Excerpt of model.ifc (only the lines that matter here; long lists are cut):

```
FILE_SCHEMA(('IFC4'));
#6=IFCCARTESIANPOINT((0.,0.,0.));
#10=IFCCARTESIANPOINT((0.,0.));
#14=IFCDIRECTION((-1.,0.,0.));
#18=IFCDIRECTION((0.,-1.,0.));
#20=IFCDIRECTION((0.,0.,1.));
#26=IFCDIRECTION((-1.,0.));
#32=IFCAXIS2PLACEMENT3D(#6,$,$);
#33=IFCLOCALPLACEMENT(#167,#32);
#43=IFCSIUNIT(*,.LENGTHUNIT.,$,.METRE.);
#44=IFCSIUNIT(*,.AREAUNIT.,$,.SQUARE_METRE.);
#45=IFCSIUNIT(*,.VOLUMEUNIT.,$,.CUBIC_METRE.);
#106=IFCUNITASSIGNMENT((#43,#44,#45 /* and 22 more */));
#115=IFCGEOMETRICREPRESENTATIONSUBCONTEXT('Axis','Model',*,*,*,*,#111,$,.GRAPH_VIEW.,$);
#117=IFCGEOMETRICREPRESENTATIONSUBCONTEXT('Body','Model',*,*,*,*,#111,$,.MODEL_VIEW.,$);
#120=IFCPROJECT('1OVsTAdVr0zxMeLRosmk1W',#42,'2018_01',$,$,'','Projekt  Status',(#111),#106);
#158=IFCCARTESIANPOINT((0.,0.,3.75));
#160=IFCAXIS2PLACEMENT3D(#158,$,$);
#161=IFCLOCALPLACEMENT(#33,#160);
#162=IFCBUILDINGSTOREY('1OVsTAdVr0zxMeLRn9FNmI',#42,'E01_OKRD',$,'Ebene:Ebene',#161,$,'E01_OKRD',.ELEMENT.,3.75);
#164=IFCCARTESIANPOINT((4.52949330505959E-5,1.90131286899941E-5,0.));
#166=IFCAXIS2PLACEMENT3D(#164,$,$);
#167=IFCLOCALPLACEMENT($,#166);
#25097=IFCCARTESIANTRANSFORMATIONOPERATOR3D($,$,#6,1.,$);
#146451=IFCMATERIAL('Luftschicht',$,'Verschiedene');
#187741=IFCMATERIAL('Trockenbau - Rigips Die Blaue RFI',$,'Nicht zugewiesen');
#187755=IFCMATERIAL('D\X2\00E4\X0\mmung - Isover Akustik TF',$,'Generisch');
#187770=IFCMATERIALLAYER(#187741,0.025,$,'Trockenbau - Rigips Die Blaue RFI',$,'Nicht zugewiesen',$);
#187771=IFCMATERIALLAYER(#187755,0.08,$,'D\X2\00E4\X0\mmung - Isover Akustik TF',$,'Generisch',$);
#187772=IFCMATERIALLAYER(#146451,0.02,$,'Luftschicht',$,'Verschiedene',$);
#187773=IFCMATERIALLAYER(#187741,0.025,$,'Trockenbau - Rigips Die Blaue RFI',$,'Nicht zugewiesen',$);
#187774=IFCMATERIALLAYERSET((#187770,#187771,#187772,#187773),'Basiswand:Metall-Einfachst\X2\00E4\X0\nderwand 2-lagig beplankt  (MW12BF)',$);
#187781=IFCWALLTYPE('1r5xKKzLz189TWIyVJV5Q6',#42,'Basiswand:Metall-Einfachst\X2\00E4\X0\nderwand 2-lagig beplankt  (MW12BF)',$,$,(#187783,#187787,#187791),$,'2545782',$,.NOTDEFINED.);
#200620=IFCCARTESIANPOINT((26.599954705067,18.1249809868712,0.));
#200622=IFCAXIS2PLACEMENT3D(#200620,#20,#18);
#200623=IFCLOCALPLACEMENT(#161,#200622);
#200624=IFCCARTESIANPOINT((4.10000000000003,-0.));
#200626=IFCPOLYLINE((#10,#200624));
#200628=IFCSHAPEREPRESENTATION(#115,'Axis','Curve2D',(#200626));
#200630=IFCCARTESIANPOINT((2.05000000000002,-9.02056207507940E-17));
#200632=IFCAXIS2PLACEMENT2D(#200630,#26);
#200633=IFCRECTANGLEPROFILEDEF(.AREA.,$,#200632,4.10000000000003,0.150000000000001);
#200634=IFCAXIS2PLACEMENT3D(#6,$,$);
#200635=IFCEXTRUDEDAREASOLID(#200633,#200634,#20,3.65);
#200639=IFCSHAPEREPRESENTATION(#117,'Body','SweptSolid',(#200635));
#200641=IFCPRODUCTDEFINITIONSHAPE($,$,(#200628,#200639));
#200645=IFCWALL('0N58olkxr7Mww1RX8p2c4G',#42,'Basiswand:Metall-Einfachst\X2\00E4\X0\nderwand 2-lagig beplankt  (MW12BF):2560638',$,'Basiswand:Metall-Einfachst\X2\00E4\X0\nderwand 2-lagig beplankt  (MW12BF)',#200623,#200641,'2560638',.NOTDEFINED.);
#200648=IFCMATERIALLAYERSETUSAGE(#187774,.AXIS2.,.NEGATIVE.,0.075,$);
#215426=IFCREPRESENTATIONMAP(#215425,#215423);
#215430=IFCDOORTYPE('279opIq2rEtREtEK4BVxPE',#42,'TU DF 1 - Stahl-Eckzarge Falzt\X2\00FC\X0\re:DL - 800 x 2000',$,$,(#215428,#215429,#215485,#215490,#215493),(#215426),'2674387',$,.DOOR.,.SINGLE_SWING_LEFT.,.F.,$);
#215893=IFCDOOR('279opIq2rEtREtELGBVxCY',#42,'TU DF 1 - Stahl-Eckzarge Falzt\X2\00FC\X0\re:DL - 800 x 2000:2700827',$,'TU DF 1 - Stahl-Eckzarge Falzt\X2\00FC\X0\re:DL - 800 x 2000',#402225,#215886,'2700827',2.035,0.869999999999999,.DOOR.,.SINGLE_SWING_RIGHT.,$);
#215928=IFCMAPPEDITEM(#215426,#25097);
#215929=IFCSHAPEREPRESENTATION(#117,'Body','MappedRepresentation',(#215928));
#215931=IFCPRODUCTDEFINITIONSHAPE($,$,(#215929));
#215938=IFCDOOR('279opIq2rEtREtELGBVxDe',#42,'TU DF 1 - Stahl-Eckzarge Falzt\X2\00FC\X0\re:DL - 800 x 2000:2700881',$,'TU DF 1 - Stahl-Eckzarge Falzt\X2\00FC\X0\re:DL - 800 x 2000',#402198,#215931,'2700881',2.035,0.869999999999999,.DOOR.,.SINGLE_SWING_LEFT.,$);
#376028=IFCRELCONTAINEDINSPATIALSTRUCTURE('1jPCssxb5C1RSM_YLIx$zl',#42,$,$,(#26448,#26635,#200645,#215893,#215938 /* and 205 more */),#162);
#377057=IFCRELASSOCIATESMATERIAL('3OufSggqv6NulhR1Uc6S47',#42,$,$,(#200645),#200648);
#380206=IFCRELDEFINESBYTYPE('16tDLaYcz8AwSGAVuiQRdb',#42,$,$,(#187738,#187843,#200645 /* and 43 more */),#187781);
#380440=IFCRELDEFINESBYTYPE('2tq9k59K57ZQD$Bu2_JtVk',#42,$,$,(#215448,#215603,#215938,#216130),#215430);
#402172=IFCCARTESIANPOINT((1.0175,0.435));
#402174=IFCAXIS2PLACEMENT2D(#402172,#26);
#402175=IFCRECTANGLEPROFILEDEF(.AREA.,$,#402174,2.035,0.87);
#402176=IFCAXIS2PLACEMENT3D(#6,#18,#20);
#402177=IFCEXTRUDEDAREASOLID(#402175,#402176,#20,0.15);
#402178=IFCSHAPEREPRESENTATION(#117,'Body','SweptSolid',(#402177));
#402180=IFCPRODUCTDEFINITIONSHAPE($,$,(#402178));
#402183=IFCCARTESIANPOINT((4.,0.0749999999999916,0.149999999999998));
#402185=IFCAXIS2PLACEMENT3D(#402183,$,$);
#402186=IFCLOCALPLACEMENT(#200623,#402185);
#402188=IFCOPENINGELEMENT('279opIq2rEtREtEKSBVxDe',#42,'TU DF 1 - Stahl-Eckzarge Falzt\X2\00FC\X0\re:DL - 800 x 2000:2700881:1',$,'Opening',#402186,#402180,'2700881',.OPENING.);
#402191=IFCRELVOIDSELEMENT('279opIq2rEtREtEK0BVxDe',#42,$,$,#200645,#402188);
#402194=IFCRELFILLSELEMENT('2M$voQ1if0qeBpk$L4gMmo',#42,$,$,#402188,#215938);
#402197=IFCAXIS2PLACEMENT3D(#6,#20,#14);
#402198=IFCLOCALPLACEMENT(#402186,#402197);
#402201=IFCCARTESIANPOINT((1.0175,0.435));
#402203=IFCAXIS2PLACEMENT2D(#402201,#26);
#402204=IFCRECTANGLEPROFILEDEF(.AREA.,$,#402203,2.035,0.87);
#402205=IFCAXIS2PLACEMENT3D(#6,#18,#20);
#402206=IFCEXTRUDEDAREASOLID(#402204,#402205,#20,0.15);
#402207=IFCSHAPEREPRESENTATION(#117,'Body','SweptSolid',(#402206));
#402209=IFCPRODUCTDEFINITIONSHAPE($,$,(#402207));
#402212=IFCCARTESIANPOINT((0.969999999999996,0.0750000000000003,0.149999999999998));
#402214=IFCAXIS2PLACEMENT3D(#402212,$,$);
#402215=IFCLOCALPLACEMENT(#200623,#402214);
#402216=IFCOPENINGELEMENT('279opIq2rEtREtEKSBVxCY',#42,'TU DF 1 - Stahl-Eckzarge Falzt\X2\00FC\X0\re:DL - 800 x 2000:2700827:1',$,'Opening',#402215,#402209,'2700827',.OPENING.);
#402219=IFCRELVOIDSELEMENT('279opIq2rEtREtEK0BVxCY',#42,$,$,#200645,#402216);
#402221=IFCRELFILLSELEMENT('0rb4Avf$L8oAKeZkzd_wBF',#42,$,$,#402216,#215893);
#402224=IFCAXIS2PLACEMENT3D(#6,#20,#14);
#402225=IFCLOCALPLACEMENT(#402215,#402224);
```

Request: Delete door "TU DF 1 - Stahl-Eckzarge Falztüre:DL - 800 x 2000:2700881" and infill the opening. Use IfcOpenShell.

```python
import ifcopenshell
import ifcopenshell.api.feature
import ifcopenshell.api.root
import ifcopenshell.geom
import ifcopenshell.util.shape

model = ifcopenshell.open("model.ifc")
settings = ifcopenshell.geom.settings()


def volume(element):
    """Net volume in cubic metres, openings subtracted."""
    shape = ifcopenshell.geom.create_shape(settings, element)
    return ifcopenshell.util.shape.get_volume(shape.geometry)


door = model.by_guid("279opIq2rEtREtELGBVxDe")
opening = door.FillsVoids[0].RelatingOpeningElement
wall = opening.VoidsElements[0].RelatingBuildingElement
before = volume(wall)

ifcopenshell.api.root.remove_product(model, product=door)
ifcopenshell.api.feature.remove_feature(model, feature=opening)

after = volume(wall)

print(f"wall volume {before:.3f} -> {after:.3f} m3")

model.write("model_v2.ifc")
```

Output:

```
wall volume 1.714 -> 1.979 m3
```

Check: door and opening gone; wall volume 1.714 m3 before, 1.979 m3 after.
